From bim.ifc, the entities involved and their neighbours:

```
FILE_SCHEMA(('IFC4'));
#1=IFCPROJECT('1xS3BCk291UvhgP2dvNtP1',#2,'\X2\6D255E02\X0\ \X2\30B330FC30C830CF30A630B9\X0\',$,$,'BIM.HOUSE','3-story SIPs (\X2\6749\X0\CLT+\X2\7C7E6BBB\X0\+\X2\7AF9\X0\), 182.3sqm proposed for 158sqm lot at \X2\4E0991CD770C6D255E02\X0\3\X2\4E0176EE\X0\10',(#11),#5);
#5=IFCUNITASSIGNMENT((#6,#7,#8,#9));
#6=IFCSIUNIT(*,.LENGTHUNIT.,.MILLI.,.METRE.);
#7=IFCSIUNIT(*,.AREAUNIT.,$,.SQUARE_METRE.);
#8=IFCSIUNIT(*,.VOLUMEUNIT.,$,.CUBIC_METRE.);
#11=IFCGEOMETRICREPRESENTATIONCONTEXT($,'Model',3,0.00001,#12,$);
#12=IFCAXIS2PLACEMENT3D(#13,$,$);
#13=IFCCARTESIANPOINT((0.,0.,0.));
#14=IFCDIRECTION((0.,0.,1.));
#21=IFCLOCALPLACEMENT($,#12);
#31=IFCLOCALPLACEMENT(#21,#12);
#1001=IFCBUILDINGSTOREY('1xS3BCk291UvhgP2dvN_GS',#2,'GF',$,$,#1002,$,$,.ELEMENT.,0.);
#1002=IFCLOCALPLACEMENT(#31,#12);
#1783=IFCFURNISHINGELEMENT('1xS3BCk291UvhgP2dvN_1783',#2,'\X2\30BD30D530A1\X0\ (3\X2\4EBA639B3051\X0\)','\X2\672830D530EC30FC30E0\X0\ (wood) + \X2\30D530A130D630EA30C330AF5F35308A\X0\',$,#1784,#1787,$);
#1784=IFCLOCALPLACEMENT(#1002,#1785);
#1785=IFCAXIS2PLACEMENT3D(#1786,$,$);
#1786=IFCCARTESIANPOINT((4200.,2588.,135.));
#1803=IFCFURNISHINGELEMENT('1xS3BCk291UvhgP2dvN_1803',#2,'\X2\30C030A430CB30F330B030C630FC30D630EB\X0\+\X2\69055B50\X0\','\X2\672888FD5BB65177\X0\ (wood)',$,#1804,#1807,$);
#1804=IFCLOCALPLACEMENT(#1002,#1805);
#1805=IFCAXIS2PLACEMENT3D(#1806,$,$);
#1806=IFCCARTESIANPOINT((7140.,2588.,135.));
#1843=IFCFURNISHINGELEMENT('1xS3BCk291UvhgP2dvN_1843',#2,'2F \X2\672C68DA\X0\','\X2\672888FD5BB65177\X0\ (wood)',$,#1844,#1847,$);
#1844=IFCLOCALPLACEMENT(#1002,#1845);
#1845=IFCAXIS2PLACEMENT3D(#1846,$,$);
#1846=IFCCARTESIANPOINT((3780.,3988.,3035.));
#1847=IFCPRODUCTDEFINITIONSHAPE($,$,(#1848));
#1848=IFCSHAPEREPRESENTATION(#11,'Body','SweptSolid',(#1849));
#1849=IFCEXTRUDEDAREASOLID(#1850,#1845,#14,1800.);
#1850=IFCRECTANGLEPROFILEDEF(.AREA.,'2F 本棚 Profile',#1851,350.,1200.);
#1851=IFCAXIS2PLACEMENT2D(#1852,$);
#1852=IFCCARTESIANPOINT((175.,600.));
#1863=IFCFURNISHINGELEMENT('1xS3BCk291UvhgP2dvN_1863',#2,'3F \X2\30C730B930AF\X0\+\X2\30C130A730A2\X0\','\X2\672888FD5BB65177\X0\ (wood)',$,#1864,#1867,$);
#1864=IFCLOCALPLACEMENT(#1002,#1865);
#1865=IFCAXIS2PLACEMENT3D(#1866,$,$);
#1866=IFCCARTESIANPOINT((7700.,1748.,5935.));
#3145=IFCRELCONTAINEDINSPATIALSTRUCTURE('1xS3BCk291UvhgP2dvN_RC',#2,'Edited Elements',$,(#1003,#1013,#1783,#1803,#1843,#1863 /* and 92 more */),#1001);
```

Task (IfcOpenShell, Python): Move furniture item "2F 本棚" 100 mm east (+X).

```python
import ifcopenshell
import ifcopenshell.api.geometry
import ifcopenshell.util.placement

model = ifcopenshell.open("bim.ifc")

item = model.by_id(1843)
matrix = ifcopenshell.util.placement.get_local_placement(item.ObjectPlacement)
matrix[0, 3] += 100.0
ifcopenshell.api.geometry.edit_object_placement(model, product=item, matrix=matrix, is_si=False)

print(ifcopenshell.util.placement.get_local_placement(item.ObjectPlacement).round(3) + 0.0)

model.write("bim_updated.ifc")
```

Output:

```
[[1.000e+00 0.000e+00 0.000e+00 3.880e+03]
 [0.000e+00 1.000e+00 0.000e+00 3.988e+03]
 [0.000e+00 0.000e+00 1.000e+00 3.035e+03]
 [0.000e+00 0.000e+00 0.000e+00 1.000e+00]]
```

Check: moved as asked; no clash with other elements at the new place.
